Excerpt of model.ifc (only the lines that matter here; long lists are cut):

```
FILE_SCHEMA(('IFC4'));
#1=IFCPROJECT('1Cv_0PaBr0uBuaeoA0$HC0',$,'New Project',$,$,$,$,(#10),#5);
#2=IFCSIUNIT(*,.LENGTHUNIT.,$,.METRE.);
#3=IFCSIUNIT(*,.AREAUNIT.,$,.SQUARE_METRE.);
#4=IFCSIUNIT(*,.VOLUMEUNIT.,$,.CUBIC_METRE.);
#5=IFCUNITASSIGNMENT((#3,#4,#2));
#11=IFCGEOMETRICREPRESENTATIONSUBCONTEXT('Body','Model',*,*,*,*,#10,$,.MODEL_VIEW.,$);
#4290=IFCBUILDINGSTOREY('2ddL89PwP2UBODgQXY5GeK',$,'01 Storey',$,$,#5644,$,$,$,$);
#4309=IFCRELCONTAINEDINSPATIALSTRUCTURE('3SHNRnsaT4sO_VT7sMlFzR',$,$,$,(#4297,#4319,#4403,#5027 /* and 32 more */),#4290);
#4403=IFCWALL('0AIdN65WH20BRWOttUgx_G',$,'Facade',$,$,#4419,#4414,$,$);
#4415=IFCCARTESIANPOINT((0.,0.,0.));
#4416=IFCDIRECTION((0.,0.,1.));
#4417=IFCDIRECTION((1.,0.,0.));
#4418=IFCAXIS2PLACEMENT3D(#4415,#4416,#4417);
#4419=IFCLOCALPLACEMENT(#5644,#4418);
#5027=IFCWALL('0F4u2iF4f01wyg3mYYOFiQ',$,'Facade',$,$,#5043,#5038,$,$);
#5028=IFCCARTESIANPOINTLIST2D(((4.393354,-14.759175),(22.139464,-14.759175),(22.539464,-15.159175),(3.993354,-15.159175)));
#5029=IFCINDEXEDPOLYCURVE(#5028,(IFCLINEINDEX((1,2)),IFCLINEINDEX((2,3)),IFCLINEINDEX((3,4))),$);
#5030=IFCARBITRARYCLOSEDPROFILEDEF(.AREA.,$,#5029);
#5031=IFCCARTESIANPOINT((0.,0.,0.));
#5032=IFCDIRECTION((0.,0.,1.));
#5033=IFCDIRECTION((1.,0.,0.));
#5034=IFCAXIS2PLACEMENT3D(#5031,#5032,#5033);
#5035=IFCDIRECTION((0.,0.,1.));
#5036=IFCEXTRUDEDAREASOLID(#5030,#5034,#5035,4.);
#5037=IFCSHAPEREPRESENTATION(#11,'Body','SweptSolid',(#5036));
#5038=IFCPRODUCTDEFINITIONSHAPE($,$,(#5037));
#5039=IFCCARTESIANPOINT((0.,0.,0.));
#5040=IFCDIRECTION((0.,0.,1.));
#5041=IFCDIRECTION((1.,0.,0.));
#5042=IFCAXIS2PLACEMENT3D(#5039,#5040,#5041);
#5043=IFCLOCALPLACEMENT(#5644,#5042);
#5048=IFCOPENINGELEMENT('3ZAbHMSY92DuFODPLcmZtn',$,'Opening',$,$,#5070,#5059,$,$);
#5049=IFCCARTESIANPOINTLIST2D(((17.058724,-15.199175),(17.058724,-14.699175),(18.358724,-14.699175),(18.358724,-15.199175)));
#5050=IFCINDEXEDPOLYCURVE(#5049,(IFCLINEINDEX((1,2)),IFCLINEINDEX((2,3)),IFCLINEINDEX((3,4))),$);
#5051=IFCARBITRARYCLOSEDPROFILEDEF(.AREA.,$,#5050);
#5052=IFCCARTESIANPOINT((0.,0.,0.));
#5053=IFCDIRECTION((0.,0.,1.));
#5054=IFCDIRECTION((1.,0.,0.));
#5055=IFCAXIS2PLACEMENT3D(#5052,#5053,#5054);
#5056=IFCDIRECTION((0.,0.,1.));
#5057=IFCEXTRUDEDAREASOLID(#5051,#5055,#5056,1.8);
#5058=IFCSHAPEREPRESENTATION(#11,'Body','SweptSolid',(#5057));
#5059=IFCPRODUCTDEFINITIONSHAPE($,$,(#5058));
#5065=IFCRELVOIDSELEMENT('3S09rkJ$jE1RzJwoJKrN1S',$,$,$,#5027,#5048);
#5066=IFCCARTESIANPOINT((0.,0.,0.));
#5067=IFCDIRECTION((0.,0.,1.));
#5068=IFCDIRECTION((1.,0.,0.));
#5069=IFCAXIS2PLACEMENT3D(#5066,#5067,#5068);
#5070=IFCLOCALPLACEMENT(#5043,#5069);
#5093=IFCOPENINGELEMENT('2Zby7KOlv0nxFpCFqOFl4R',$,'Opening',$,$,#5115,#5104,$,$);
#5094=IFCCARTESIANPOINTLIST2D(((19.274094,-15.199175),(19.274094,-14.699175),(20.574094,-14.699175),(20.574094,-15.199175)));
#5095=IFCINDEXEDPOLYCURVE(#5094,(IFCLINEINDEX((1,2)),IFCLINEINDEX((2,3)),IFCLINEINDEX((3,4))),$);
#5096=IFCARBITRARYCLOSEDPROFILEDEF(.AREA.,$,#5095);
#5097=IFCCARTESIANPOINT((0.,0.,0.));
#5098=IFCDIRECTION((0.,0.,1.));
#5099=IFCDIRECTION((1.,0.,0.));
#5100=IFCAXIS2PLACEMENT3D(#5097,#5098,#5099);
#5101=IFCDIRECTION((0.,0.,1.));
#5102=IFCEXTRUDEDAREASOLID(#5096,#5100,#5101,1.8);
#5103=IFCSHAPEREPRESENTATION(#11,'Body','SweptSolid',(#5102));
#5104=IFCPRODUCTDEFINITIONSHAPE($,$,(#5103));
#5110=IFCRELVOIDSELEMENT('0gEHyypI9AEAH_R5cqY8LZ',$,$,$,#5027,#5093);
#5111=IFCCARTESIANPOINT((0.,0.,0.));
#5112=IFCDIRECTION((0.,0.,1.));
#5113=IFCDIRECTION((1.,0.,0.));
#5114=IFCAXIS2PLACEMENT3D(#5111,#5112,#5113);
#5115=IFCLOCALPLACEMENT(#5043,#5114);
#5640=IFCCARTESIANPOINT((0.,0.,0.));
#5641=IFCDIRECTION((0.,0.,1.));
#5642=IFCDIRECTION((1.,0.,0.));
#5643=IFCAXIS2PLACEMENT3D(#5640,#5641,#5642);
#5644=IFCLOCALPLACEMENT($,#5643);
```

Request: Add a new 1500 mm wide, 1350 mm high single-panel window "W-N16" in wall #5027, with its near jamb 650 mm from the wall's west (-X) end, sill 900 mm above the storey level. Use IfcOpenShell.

```python
import numpy as np
import ifcopenshell
import ifcopenshell.api.feature
import ifcopenshell.api.geometry
import ifcopenshell.api.root
import ifcopenshell.api.spatial
import ifcopenshell.geom
import ifcopenshell.util.element
import ifcopenshell.util.placement
import ifcopenshell.util.representation
import ifcopenshell.util.shape
import ifcopenshell.util.unit

model = ifcopenshell.open("model.ifc")
unit_scale = ifcopenshell.util.unit.calculate_unit_scale(model)
settings = ifcopenshell.geom.settings()


def volume(element):
    """Net volume in cubic metres, openings subtracted."""
    shape = ifcopenshell.geom.create_shape(settings, element)
    return ifcopenshell.util.shape.get_volume(shape.geometry)


wall = model.by_guid("0F4u2iF4f01wyg3mYYOFiQ")
storey = ifcopenshell.util.element.get_container(wall, ifc_class="IfcBuildingStorey")
context = ifcopenshell.util.representation.get_context(model, "Model", "Body", "MODEL_VIEW")
before = volume(wall)

width, height, from_end, sill = 1.5, 1.35, 0.65, 0.9  # metres

# The wall runs along its own X axis, and the end named is its -X end.
wall_shape = ifcopenshell.geom.create_shape(settings, wall)
x, y, z = ifcopenshell.util.shape.get_vertices(wall_shape.geometry).T
start = x.min() + from_end
face, thickness = float(y.min()), float(y.max() - y.min())
wall_matrix = ifcopenshell.util.placement.get_local_placement(wall.ObjectPlacement)
level = ifcopenshell.util.placement.get_local_placement(storey.ObjectPlacement)[2, 3]


def in_wall(x, y):
    """Placement at x, y metres in the wall's axes, at sill height."""
    matrix = wall_matrix.copy()
    matrix[:, 3] = wall_matrix @ np.array([x / unit_scale, y / unit_scale, 0.0, 1.0])
    matrix[2, 3] = level + sill / unit_scale
    return matrix


# Opening: a box that overshoots both wall faces by 50 mm.
opening = ifcopenshell.api.root.create_entity(model, ifc_class="IfcOpeningElement", predefined_type="OPENING")
box = ifcopenshell.api.geometry.add_wall_representation(
    model, context=context, length=width, height=height, thickness=thickness + 0.1
)
ifcopenshell.api.geometry.assign_representation(model, product=opening, representation=box)
ifcopenshell.api.geometry.edit_object_placement(model, product=opening, matrix=in_wall(start, face - 0.05), is_si=False)
ifcopenshell.api.feature.add_feature(model, feature=opening, element=wall)

window = ifcopenshell.api.root.create_entity(model, ifc_class="IfcWindow", name="W-N16", predefined_type="WINDOW")
window.OverallWidth, window.OverallHeight = width / unit_scale, height / unit_scale
window.PartitioningType = "SINGLE_PANEL"
body = ifcopenshell.api.geometry.add_window_representation(
    model,
    context=context,
    overall_width=window.OverallWidth,
    overall_height=window.OverallHeight,
    partition_type="SINGLE_PANEL",
)
ifcopenshell.api.geometry.assign_representation(model, product=window, representation=body)
ifcopenshell.api.spatial.assign_container(model, products=[window], relating_structure=storey)
ifcopenshell.api.feature.add_filling(model, opening=opening, element=window)

# Centre the window in the wall's thickness.
ifcopenshell.api.geometry.edit_object_placement(model, product=window, matrix=in_wall(start, face), is_si=False)
window_shape = ifcopenshell.geom.create_shape(settings, window)
depth = ifcopenshell.util.shape.get_vertices(window_shape.geometry)[:, 1]
offset = face + thickness / 2 - (depth.min() + depth.max()) / 2
ifcopenshell.api.geometry.edit_object_placement(model, product=window, matrix=in_wall(start, offset), is_si=False)

after = volume(wall)

print(f"wall volume {before:.3f} -> {after:.3f} m3")

model.write("model_edited.ifc")
```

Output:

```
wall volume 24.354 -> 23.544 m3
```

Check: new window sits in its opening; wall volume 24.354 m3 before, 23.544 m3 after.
